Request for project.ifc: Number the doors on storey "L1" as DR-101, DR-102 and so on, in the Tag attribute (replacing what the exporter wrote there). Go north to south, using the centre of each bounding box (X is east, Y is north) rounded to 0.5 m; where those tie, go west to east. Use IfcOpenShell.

First a look at what the model holds.

```python
import ifcopenshell
import ifcopenshell.util.element
import ifcopenshell.util.placement

model = ifcopenshell.open("project.ifc")
print(model.schema)
storey = next(s for s in model.by_type("IfcBuildingStorey") if s.Name == "L1")
doors = [e for e in ifcopenshell.util.element.get_decomposition(storey) if e.is_a("IfcDoor")]
for e in sorted(doors, key=lambda e: e.id()):
    origin = ifcopenshell.util.placement.get_local_placement(e.ObjectPlacement)[:3, 3]
    print(e.id(), e.Tag, e.Name, origin.round(2) + 0.0, sep=" | ")
```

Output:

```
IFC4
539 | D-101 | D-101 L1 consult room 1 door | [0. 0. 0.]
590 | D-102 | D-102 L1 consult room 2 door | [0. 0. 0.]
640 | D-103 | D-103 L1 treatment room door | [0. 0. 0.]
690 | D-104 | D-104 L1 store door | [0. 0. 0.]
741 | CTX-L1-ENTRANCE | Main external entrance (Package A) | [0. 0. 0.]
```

```python
import ifcopenshell
import ifcopenshell.geom
import ifcopenshell.util.element
import ifcopenshell.util.shape

model = ifcopenshell.open("project.ifc")
settings = ifcopenshell.geom.settings()
settings.set("use-world-coords", True)


def centre(element):
    shape = ifcopenshell.geom.create_shape(settings, element)
    return ifcopenshell.util.shape.get_bbox_centroid(shape.geometry)


storey = next(s for s in model.by_type("IfcBuildingStorey") if s.Name == "L1")
doors = [e for e in ifcopenshell.util.element.get_decomposition(storey) if e.is_a("IfcDoor")]

# Insertion points can sit at a corner or the storey origin, so sort by the geometry (in metres).
centres = {e: centre(e) for e in doors}
doors.sort(key=lambda e: (-round(centres[e][1] / 0.5), centres[e][0]))

for i, e in enumerate(doors, start=1):
    number = f"DR-1{i:02d}"
    e.Tag = number
    print(e.id(), number)

model.write("project-out.ifc")
```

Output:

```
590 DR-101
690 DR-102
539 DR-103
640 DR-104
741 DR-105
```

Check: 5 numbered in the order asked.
